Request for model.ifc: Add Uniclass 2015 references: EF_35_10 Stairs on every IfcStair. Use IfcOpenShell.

First a look at what the model holds.

```python
import ifcopenshell

model = ifcopenshell.open("model.ifc")
print(model.schema)
print("classifications:", [c.Name for c in model.by_type("IfcClassification")])
for ifc_class in ("IfcDoor", "IfcRoof", "IfcStair", "IfcWall", "IfcWindow"):
    print(ifc_class, len(model.by_type(ifc_class)))
```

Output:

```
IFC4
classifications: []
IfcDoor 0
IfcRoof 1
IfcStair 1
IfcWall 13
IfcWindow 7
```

```python
import ifcopenshell
import ifcopenshell.api.classification

model = ifcopenshell.open("model.ifc")

system = ifcopenshell.api.classification.add_classification(model, classification="Uniclass 2015")

codes = {
    "IfcStair": ("EF_35_10", "Stairs"),
}
for ifc_class, (code, name) in codes.items():
    products = model.by_type(ifc_class)
    ifcopenshell.api.classification.add_reference(
        model, products=products, classification=system, identification=code, name=name
    )
    print(code, len(products))

model.write("model_rev.ifc")
```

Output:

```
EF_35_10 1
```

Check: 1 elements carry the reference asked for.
